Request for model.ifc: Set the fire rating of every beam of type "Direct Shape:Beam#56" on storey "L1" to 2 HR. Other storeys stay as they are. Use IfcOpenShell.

First a look at what the model holds.

```python
import ifcopenshell
import ifcopenshell.util.element

model = ifcopenshell.open("model.ifc")
print(model.schema)
storey = next(s for s in model.by_type("IfcBuildingStorey") if s.Name == "L1")
beams = [e for e in ifcopenshell.util.element.get_decomposition(storey) if e.is_a("IfcBeam")]
seen = {}
for e in beams:
    element_type = ifcopenshell.util.element.get_type(e)
    key = (element_type.Name if element_type != e and element_type else None, ifcopenshell.util.element.get_pset(e, "Pset_BeamCommon", "FireRating"))
    seen[key] = seen.get(key, 0) + 1
for (name, value), count in sorted(seen.items(), key=str):
    print(count, "x", name, "|", value)
```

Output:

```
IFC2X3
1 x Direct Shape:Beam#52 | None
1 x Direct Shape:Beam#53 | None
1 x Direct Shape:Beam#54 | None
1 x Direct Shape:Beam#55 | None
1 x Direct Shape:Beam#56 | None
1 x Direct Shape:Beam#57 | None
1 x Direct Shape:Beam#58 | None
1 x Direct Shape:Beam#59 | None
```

```python
import ifcopenshell
import ifcopenshell.api.pset
import ifcopenshell.util.element

model = ifcopenshell.open("model.ifc")

storey = next(s for s in model.by_type("IfcBuildingStorey") if s.Name == "L1")
beams = [e for e in ifcopenshell.util.element.get_decomposition(storey) if e.is_a("IfcBeam")]

count = 0
for e in beams:
    element_type = ifcopenshell.util.element.get_type(e)
    if element_type in (None, e) or element_type.Name != "Direct Shape:Beam#56":
        continue
    # add_pset returns the element's existing set when there is one.
    pset = ifcopenshell.api.pset.add_pset(model, product=e, name="Pset_BeamCommon")
    ifcopenshell.api.pset.edit_pset(model, pset=pset, properties={"FireRating": "2 HR"})
    count += 1

print(count, "beams updated")

model.write("model_edited.ifc")
```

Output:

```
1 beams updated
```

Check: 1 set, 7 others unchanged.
